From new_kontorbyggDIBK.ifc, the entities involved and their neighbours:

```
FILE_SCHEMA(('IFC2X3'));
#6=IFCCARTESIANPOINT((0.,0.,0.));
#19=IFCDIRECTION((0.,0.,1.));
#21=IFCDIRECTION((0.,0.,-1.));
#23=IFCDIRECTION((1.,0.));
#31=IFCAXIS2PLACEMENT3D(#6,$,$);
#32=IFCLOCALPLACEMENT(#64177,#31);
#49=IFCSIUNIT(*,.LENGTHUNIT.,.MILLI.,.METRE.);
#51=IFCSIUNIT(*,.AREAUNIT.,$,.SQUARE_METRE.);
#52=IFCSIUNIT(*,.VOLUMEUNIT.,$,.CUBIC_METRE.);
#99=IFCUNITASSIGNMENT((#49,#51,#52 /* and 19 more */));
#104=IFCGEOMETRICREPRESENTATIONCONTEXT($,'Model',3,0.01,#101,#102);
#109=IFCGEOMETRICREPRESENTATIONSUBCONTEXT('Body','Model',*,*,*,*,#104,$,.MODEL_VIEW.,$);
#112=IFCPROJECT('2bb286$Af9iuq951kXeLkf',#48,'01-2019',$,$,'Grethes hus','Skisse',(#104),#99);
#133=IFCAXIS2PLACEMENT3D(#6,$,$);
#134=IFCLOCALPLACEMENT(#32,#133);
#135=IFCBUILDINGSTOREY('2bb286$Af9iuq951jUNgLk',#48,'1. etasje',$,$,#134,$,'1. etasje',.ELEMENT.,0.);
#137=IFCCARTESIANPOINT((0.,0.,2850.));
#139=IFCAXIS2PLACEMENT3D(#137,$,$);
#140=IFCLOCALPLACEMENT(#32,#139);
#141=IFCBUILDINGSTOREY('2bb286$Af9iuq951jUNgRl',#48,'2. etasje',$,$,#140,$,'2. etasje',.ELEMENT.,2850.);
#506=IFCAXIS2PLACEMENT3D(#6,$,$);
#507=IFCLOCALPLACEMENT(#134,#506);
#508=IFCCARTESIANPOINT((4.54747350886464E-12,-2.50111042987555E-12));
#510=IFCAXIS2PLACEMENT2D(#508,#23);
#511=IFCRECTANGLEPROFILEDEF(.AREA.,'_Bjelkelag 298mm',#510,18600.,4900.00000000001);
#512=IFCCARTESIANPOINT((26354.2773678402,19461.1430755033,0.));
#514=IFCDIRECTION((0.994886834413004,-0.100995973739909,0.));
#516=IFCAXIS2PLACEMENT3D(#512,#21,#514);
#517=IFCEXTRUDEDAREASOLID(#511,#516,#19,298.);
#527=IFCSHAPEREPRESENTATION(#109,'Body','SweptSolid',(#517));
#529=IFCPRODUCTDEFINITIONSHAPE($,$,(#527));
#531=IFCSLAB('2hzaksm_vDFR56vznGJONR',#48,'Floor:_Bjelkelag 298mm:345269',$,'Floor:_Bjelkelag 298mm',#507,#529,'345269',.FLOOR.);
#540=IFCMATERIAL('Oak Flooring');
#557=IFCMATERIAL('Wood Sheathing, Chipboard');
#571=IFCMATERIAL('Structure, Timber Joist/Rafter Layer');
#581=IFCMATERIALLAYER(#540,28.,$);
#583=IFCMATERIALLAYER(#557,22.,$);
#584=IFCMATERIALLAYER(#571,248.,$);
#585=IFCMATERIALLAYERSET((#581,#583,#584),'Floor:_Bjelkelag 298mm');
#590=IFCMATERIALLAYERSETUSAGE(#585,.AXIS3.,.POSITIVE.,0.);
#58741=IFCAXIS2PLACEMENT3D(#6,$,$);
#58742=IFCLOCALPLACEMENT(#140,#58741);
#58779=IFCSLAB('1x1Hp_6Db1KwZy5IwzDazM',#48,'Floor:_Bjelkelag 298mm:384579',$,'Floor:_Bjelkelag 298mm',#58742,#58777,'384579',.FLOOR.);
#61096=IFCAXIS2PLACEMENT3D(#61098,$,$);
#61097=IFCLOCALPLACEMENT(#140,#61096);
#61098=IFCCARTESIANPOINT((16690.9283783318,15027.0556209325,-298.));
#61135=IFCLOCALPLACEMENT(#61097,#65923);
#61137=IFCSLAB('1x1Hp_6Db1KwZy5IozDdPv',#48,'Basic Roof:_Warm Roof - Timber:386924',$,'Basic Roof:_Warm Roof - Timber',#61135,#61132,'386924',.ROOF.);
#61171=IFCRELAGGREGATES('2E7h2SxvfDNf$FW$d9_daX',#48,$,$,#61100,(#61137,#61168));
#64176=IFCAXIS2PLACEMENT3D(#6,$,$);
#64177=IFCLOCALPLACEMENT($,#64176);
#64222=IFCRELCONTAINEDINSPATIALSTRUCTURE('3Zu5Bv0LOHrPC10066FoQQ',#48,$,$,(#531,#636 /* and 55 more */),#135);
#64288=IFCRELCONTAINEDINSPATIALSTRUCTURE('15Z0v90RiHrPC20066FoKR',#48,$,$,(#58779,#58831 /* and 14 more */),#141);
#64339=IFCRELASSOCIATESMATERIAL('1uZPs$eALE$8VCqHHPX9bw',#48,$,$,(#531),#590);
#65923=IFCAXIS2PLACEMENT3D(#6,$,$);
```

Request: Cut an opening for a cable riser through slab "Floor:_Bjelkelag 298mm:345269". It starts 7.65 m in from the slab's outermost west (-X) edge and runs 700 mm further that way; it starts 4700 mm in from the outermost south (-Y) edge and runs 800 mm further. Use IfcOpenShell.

```python
import numpy as np
import ifcopenshell
import ifcopenshell.api.feature
import ifcopenshell.api.geometry
import ifcopenshell.api.root
import ifcopenshell.geom
import ifcopenshell.util.placement
import ifcopenshell.util.representation
import ifcopenshell.util.shape
import ifcopenshell.util.unit

model = ifcopenshell.open("new_kontorbyggDIBK.ifc")
unit_scale = ifcopenshell.util.unit.calculate_unit_scale(model)
settings = ifcopenshell.geom.settings()


def volume(element):
    """Net volume in cubic metres, openings subtracted."""
    shape = ifcopenshell.geom.create_shape(settings, element)
    return ifcopenshell.util.shape.get_volume(shape.geometry)


slab = model.by_guid("2hzaksm_vDFR56vznGJONR")
before = volume(slab)

# Extent in the slab's own axes, in metres. The edges named are its -X and -Y sides.
slab_shape = ifcopenshell.geom.create_shape(settings, slab)
vertices = ifcopenshell.util.shape.get_vertices(slab_shape.geometry)
x_min, y_min, bottom = vertices.min(axis=0)
top = vertices[:, 2].max()

opening = ifcopenshell.api.root.create_entity(model, ifc_class="IfcOpeningElement", name="Cable riser opening")
context = ifcopenshell.util.representation.get_context(model, "Model", "Body", "MODEL_VIEW")
width, depth = 0.7, 0.8
outline = [(0.0, 0.0), (width, 0.0), (width, depth), (0.0, depth), (0.0, 0.0)]
# Overshoot both faces by 50 mm so the cut is clean.
shape = ifcopenshell.api.geometry.add_slab_representation(
    model, context=context, depth=top - bottom + 0.1, polyline=outline
)
ifcopenshell.api.geometry.assign_representation(model, product=opening, representation=shape)

matrix = ifcopenshell.util.placement.get_local_placement(slab.ObjectPlacement)
matrix[:, 3] = matrix @ np.append(np.array([x_min + 7.65, y_min + 4.7, bottom - 0.05]) / unit_scale, 1.0)
ifcopenshell.api.geometry.edit_object_placement(model, product=opening, matrix=matrix, is_si=False)
ifcopenshell.api.feature.add_feature(model, feature=opening, element=slab)

after = volume(slab)

print(f"slab volume {before:.3f} -> {after:.3f} m3")

model.write("new_kontorbyggDIBK_rev.ifc")
```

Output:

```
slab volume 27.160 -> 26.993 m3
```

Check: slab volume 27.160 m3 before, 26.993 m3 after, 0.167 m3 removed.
